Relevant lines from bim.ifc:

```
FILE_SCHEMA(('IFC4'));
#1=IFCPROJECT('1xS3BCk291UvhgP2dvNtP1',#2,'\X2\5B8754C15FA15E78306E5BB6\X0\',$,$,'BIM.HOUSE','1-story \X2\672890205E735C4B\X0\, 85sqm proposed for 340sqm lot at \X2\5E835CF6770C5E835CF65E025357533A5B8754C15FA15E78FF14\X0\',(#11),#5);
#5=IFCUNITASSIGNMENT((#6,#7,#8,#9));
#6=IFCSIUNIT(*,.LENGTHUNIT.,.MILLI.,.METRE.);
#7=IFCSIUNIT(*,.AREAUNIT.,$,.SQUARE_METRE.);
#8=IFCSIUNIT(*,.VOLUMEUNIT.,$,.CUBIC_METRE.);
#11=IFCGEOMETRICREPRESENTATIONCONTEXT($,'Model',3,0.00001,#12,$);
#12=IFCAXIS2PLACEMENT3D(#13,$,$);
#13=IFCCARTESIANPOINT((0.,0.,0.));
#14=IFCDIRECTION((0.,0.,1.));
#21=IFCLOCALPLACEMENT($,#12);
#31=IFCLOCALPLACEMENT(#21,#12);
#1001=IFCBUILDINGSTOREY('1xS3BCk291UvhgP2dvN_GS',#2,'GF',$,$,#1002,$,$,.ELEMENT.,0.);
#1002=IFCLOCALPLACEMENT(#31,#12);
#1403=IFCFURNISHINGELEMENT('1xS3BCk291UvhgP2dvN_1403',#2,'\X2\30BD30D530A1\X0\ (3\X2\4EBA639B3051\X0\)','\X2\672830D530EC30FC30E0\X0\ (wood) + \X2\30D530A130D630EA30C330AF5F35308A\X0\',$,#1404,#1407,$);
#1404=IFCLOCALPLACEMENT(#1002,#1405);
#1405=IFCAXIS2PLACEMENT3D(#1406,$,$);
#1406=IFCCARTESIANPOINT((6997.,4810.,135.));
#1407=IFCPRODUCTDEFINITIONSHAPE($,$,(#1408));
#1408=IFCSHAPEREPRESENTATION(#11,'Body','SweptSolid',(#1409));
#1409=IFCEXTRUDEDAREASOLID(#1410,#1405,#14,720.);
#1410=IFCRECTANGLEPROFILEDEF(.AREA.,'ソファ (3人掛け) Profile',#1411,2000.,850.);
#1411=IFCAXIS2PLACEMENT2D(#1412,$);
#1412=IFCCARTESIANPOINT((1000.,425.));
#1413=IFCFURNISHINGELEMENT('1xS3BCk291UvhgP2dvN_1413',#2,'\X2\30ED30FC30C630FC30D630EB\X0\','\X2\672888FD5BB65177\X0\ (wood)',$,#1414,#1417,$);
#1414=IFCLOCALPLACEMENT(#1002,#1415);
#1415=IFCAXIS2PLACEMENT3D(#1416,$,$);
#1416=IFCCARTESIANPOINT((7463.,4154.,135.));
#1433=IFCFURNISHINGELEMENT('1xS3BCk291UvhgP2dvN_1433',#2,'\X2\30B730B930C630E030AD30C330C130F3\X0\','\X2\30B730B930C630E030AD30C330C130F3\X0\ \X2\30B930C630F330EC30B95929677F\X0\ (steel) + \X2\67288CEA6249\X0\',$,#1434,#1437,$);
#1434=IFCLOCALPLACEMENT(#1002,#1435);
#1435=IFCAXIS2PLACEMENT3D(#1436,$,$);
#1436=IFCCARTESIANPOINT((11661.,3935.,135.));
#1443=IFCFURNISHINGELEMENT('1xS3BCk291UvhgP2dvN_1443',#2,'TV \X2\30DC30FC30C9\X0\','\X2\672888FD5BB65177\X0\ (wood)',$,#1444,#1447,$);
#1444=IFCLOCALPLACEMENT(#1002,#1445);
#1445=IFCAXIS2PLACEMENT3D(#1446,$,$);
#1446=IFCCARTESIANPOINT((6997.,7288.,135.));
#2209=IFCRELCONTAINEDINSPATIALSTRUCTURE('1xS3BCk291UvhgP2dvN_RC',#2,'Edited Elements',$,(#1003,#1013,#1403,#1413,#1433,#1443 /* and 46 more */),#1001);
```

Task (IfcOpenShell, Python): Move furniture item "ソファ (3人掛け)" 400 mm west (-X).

```python
import ifcopenshell
import ifcopenshell.api.geometry
import ifcopenshell.util.placement
import ifcopenshell.util.unit

model = ifcopenshell.open("bim.ifc")
unit_scale = ifcopenshell.util.unit.calculate_unit_scale(model)

item = model.by_id(1403)
matrix = ifcopenshell.util.placement.get_local_placement(item.ObjectPlacement)
matrix[0, 3] -= 0.4 / unit_scale
ifcopenshell.api.geometry.edit_object_placement(model, product=item, matrix=matrix, is_si=False)

print(ifcopenshell.util.placement.get_local_placement(item.ObjectPlacement).round(3) + 0.0)

model.write("bim_v2.ifc")
```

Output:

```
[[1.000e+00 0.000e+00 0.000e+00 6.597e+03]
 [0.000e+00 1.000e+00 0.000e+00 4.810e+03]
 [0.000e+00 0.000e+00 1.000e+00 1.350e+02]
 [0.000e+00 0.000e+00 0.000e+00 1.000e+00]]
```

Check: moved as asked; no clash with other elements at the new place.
